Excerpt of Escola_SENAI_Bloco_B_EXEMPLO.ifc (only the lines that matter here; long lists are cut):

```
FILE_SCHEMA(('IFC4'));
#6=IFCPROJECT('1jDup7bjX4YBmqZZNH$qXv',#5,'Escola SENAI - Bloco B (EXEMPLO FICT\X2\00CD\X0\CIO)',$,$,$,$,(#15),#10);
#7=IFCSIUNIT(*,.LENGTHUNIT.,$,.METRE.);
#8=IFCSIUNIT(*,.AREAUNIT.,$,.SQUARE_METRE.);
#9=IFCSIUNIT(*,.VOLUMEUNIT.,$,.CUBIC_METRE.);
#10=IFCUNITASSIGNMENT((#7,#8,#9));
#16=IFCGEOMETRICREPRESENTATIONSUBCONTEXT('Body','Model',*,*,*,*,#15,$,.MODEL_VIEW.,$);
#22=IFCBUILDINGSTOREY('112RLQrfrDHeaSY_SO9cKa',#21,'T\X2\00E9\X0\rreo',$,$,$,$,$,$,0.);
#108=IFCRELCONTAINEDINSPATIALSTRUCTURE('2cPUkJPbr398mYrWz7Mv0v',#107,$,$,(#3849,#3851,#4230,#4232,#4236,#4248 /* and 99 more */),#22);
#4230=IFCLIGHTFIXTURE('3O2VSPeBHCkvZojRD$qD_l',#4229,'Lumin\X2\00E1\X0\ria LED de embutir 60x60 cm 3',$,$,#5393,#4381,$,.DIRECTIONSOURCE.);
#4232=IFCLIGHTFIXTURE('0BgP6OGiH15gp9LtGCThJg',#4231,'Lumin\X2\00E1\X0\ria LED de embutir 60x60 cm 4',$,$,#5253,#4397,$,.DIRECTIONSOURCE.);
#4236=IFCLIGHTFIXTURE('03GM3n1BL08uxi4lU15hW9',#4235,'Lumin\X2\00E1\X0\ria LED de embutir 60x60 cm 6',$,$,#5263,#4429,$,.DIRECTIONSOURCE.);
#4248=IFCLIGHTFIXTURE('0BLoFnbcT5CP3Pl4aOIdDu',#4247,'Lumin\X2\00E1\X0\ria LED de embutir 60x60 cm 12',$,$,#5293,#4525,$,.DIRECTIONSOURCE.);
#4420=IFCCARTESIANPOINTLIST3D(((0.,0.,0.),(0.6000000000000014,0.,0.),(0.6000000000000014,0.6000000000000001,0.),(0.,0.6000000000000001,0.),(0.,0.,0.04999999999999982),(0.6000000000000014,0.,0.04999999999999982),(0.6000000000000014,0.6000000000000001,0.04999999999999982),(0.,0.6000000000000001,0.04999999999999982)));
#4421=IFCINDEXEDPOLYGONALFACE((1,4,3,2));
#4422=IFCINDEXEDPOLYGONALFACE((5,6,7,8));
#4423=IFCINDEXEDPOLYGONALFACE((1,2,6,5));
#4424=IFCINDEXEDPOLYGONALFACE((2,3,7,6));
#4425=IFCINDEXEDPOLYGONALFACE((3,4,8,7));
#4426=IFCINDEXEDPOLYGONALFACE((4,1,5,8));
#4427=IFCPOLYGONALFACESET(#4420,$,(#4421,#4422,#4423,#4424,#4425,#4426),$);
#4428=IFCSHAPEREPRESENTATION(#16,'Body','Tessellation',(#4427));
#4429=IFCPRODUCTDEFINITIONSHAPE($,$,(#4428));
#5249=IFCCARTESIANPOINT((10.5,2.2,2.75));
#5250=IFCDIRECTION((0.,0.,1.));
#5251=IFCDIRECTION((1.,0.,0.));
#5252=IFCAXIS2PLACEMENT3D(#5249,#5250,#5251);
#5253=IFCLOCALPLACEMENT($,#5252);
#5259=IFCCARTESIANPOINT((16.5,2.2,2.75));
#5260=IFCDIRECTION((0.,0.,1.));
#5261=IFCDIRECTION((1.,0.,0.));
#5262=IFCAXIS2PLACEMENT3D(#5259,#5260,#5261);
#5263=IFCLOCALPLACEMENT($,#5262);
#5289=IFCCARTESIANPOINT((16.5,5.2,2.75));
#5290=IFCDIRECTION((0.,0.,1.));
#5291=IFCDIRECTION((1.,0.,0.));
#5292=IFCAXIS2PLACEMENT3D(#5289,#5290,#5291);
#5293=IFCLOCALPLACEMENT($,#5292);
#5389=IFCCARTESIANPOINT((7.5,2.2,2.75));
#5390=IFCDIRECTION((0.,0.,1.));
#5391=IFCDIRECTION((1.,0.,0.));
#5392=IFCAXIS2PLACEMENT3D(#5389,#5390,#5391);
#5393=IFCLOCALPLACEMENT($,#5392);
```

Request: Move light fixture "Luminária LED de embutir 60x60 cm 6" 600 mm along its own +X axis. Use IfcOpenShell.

```python
import ifcopenshell
import ifcopenshell.api.geometry
import ifcopenshell.util.placement
import ifcopenshell.util.unit

model = ifcopenshell.open("Escola_SENAI_Bloco_B_EXEMPLO.ifc")
unit_scale = ifcopenshell.util.unit.calculate_unit_scale(model)

item = model.by_id(4236)
matrix = ifcopenshell.util.placement.get_local_placement(item.ObjectPlacement)
matrix[:3, 3] += matrix[:3, 0] * 0.6 / unit_scale
ifcopenshell.api.geometry.edit_object_placement(model, product=item, matrix=matrix, is_si=False)

print(ifcopenshell.util.placement.get_local_placement(item.ObjectPlacement).round(3) + 0.0)

model.write("Escola_SENAI_Bloco_B_EXEMPLO_edited.ifc")
```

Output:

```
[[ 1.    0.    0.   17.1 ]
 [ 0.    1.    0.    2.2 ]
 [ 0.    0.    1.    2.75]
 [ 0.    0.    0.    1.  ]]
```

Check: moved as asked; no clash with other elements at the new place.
